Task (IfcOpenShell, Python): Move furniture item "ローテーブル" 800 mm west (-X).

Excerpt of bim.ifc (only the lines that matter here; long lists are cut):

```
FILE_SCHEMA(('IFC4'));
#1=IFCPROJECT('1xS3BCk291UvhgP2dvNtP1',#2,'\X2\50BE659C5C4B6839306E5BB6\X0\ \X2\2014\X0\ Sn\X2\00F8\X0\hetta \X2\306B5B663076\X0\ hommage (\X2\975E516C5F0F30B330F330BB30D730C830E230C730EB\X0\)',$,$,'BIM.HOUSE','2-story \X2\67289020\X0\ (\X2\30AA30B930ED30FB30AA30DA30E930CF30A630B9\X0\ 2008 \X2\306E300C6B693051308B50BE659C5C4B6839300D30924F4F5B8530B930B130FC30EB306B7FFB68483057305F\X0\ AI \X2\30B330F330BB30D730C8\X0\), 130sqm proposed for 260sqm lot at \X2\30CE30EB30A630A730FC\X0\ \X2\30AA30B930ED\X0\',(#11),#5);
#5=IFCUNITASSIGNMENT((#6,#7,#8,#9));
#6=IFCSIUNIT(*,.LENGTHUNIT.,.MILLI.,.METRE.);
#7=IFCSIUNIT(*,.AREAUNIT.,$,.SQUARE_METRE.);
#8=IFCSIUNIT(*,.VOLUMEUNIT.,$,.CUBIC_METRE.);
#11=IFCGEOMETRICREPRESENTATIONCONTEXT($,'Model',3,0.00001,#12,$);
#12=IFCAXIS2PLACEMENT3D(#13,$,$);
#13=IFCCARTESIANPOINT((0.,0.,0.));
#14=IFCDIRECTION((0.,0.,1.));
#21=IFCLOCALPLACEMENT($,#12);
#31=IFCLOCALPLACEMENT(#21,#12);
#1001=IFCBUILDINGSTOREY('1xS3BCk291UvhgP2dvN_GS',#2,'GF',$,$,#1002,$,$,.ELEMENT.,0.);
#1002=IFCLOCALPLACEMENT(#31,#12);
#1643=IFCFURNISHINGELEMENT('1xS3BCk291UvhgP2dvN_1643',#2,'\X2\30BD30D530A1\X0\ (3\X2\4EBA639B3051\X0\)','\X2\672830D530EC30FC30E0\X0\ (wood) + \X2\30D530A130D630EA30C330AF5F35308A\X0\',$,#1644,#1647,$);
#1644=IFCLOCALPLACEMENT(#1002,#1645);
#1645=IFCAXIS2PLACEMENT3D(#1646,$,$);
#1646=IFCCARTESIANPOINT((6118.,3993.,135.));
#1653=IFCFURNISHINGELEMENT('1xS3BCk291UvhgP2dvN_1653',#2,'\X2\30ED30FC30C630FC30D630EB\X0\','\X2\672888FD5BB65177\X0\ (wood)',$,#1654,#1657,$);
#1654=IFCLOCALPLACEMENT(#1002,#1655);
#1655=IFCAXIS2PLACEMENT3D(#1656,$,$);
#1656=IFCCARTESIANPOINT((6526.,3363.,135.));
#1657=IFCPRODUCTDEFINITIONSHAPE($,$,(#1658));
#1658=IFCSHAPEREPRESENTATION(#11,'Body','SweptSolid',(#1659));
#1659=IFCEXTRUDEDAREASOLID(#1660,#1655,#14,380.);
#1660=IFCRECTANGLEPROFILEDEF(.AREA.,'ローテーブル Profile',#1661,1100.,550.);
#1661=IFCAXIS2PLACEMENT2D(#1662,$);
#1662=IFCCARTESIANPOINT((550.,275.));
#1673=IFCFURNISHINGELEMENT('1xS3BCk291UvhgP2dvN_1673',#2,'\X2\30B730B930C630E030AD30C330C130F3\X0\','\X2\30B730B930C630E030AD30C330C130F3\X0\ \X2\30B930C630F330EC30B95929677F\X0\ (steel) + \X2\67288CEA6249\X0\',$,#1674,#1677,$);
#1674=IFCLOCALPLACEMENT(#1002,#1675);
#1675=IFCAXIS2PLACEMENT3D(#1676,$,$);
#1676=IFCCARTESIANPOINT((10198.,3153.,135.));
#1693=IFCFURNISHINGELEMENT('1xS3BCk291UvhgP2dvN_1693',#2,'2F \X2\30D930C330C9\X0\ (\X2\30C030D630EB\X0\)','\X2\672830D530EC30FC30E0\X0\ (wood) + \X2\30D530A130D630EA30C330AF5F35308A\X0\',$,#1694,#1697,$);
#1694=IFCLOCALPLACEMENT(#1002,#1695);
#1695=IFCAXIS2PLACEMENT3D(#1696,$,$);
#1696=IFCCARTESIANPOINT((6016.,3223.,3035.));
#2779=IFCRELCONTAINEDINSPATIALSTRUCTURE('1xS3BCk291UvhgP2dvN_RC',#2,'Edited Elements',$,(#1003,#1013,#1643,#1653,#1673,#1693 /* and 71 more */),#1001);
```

```python
import ifcopenshell
import ifcopenshell.api.geometry
import ifcopenshell.util.placement
import ifcopenshell.util.unit

model = ifcopenshell.open("bim.ifc")
unit_scale = ifcopenshell.util.unit.calculate_unit_scale(model)

item = model.by_guid("1xS3BCk291UvhgP2dvN_1653")
matrix = ifcopenshell.util.placement.get_local_placement(item.ObjectPlacement)
matrix[0, 3] -= 0.8 / unit_scale
ifcopenshell.api.geometry.edit_object_placement(model, product=item, matrix=matrix, is_si=False)

print(ifcopenshell.util.placement.get_local_placement(item.ObjectPlacement).round(3) + 0.0)

model.write("bim_rev.ifc")
```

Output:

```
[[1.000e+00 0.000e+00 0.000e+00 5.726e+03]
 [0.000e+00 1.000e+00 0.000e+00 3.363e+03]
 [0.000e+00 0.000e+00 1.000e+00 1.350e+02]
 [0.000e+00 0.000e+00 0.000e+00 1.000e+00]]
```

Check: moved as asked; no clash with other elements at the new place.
